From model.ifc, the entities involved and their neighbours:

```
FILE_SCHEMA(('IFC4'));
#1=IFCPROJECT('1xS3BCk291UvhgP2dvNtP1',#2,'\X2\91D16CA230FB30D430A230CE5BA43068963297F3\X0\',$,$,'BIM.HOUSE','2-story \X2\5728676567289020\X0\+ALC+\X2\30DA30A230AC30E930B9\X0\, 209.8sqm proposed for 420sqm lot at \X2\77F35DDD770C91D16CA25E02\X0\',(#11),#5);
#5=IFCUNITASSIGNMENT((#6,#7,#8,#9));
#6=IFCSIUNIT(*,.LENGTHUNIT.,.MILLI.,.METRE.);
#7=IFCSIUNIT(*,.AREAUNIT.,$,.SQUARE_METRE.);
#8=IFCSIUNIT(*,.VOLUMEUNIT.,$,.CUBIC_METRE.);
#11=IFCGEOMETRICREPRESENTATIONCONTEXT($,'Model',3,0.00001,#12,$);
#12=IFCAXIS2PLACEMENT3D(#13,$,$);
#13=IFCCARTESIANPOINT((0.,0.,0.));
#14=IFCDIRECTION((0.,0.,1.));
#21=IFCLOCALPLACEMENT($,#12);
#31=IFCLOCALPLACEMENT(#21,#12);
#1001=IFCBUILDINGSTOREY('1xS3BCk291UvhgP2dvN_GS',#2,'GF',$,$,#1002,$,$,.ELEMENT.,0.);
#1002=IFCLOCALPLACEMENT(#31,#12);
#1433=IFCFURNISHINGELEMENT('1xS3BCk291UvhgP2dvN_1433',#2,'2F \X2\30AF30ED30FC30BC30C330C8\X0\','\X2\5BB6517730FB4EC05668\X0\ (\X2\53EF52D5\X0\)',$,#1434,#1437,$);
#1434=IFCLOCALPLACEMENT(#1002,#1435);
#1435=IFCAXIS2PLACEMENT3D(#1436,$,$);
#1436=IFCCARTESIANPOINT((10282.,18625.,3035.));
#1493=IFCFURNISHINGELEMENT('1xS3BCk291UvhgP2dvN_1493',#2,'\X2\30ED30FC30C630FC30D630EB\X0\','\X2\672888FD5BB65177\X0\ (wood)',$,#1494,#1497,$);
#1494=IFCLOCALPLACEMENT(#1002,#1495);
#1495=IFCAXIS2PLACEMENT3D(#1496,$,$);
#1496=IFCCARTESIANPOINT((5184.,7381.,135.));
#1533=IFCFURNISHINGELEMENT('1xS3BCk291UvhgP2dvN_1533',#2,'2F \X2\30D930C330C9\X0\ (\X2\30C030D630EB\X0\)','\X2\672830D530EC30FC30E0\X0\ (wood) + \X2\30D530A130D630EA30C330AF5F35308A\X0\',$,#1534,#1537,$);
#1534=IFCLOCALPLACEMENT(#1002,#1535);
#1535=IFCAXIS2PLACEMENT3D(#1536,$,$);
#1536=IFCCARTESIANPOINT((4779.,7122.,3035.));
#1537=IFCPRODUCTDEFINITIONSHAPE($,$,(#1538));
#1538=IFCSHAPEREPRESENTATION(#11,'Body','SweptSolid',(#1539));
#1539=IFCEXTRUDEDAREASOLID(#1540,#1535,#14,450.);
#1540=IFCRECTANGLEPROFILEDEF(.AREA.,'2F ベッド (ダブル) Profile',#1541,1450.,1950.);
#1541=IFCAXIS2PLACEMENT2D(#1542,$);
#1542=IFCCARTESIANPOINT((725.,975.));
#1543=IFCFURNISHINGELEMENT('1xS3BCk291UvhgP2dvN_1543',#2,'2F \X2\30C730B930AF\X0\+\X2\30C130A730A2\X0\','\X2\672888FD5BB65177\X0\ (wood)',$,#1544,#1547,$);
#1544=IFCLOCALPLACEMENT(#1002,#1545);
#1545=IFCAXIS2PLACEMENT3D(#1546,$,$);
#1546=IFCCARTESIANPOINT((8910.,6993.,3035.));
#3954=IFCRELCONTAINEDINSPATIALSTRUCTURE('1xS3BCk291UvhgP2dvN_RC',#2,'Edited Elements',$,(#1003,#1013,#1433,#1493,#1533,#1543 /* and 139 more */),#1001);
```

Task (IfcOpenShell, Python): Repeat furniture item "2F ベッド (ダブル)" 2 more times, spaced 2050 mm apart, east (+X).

```python
import numpy as np
import ifcopenshell
import ifcopenshell.api.geometry
import ifcopenshell.api.root
import ifcopenshell.util.element
import ifcopenshell.util.placement
import ifcopenshell.util.unit

model = ifcopenshell.open("model.ifc")
unit_scale = ifcopenshell.util.unit.calculate_unit_scale(model)


def reuse_history(source, copy):
    """copy_class also copies each property set's owner history, people and application; keep the originals."""
    for rel in copy.IsDefinedBy:
        if rel.is_a("IfcRelDefinesByProperties") and (history := rel.RelatingPropertyDefinition.OwnerHistory):
            rel.RelatingPropertyDefinition.OwnerHistory = source.OwnerHistory
            ifcopenshell.util.element.remove_deep2(model, history)


source = model.by_id(1533)
base = ifcopenshell.util.placement.get_local_placement(source.ObjectPlacement)
step = np.array([1.0, 0.0, 0.0]) * 2.05 / unit_scale

for i in range(1, 3):
    copy = ifcopenshell.api.root.copy_class(model, product=source)
    copy.Representation = ifcopenshell.util.element.copy_deep(
        model, source.Representation, exclude=["IfcGeometricRepresentationContext", "IfcRepresentationMap"]
    )
    reuse_history(source, copy)
    matrix = base.copy()
    matrix[:3, 3] += i * step
    print("added at", matrix[:3, 3].round(3) + 0.0)
    ifcopenshell.api.geometry.edit_object_placement(model, product=copy, matrix=matrix, is_si=False)

model.write("model_rev.ifc")
```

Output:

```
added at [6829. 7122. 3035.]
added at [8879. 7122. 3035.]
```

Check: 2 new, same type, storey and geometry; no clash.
